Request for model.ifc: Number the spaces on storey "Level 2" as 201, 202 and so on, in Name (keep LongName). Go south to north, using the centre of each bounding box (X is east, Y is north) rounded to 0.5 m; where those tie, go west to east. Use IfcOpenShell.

First a look at what the model holds.

```python
import ifcopenshell
import ifcopenshell.util.element
import ifcopenshell.util.placement

model = ifcopenshell.open("model.ifc")
print(model.schema)
storey = next(s for s in model.by_type("IfcBuildingStorey") if s.Name == "Level 2")
spaces = [e for e in ifcopenshell.util.element.get_decomposition(storey) if e.is_a("IfcSpace")]
for e in sorted(spaces, key=lambda e: e.id()):
    origin = ifcopenshell.util.placement.get_local_placement(e.ObjectPlacement)[:3, 3]
    print(e.id(), e.Name, e.LongName, origin.round(2) + 0.0, sep=" | ")
```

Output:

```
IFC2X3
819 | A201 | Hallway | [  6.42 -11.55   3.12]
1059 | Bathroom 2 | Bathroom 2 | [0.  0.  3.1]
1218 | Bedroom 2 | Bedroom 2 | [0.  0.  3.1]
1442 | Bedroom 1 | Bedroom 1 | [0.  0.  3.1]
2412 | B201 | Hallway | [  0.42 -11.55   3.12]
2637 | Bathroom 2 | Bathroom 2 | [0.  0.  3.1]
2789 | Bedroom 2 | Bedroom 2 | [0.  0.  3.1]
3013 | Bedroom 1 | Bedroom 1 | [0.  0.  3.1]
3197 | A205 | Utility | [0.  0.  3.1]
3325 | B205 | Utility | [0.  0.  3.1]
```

```python
import ifcopenshell
import ifcopenshell.geom
import ifcopenshell.util.element
import ifcopenshell.util.shape

model = ifcopenshell.open("model.ifc")
settings = ifcopenshell.geom.settings()
settings.set("use-world-coords", True)


def centre(element):
    shape = ifcopenshell.geom.create_shape(settings, element)
    return ifcopenshell.util.shape.get_bbox_centroid(shape.geometry)


storey = next(s for s in model.by_type("IfcBuildingStorey") if s.Name == "Level 2")
spaces = [e for e in ifcopenshell.util.element.get_decomposition(storey) if e.is_a("IfcSpace")]

# Insertion points can sit at a corner or the storey origin, so sort by the geometry (in metres).
centres = {e: centre(e) for e in spaces}
spaces.sort(key=lambda e: (round(centres[e][1] / 0.5), centres[e][0]))

for i, e in enumerate(spaces, start=1):
    number = f"2{i:02d}"
    e.Name = number
    print(e.id(), number)

model.write("model_edited.ifc")
```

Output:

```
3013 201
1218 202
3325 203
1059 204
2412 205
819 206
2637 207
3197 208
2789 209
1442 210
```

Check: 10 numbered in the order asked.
